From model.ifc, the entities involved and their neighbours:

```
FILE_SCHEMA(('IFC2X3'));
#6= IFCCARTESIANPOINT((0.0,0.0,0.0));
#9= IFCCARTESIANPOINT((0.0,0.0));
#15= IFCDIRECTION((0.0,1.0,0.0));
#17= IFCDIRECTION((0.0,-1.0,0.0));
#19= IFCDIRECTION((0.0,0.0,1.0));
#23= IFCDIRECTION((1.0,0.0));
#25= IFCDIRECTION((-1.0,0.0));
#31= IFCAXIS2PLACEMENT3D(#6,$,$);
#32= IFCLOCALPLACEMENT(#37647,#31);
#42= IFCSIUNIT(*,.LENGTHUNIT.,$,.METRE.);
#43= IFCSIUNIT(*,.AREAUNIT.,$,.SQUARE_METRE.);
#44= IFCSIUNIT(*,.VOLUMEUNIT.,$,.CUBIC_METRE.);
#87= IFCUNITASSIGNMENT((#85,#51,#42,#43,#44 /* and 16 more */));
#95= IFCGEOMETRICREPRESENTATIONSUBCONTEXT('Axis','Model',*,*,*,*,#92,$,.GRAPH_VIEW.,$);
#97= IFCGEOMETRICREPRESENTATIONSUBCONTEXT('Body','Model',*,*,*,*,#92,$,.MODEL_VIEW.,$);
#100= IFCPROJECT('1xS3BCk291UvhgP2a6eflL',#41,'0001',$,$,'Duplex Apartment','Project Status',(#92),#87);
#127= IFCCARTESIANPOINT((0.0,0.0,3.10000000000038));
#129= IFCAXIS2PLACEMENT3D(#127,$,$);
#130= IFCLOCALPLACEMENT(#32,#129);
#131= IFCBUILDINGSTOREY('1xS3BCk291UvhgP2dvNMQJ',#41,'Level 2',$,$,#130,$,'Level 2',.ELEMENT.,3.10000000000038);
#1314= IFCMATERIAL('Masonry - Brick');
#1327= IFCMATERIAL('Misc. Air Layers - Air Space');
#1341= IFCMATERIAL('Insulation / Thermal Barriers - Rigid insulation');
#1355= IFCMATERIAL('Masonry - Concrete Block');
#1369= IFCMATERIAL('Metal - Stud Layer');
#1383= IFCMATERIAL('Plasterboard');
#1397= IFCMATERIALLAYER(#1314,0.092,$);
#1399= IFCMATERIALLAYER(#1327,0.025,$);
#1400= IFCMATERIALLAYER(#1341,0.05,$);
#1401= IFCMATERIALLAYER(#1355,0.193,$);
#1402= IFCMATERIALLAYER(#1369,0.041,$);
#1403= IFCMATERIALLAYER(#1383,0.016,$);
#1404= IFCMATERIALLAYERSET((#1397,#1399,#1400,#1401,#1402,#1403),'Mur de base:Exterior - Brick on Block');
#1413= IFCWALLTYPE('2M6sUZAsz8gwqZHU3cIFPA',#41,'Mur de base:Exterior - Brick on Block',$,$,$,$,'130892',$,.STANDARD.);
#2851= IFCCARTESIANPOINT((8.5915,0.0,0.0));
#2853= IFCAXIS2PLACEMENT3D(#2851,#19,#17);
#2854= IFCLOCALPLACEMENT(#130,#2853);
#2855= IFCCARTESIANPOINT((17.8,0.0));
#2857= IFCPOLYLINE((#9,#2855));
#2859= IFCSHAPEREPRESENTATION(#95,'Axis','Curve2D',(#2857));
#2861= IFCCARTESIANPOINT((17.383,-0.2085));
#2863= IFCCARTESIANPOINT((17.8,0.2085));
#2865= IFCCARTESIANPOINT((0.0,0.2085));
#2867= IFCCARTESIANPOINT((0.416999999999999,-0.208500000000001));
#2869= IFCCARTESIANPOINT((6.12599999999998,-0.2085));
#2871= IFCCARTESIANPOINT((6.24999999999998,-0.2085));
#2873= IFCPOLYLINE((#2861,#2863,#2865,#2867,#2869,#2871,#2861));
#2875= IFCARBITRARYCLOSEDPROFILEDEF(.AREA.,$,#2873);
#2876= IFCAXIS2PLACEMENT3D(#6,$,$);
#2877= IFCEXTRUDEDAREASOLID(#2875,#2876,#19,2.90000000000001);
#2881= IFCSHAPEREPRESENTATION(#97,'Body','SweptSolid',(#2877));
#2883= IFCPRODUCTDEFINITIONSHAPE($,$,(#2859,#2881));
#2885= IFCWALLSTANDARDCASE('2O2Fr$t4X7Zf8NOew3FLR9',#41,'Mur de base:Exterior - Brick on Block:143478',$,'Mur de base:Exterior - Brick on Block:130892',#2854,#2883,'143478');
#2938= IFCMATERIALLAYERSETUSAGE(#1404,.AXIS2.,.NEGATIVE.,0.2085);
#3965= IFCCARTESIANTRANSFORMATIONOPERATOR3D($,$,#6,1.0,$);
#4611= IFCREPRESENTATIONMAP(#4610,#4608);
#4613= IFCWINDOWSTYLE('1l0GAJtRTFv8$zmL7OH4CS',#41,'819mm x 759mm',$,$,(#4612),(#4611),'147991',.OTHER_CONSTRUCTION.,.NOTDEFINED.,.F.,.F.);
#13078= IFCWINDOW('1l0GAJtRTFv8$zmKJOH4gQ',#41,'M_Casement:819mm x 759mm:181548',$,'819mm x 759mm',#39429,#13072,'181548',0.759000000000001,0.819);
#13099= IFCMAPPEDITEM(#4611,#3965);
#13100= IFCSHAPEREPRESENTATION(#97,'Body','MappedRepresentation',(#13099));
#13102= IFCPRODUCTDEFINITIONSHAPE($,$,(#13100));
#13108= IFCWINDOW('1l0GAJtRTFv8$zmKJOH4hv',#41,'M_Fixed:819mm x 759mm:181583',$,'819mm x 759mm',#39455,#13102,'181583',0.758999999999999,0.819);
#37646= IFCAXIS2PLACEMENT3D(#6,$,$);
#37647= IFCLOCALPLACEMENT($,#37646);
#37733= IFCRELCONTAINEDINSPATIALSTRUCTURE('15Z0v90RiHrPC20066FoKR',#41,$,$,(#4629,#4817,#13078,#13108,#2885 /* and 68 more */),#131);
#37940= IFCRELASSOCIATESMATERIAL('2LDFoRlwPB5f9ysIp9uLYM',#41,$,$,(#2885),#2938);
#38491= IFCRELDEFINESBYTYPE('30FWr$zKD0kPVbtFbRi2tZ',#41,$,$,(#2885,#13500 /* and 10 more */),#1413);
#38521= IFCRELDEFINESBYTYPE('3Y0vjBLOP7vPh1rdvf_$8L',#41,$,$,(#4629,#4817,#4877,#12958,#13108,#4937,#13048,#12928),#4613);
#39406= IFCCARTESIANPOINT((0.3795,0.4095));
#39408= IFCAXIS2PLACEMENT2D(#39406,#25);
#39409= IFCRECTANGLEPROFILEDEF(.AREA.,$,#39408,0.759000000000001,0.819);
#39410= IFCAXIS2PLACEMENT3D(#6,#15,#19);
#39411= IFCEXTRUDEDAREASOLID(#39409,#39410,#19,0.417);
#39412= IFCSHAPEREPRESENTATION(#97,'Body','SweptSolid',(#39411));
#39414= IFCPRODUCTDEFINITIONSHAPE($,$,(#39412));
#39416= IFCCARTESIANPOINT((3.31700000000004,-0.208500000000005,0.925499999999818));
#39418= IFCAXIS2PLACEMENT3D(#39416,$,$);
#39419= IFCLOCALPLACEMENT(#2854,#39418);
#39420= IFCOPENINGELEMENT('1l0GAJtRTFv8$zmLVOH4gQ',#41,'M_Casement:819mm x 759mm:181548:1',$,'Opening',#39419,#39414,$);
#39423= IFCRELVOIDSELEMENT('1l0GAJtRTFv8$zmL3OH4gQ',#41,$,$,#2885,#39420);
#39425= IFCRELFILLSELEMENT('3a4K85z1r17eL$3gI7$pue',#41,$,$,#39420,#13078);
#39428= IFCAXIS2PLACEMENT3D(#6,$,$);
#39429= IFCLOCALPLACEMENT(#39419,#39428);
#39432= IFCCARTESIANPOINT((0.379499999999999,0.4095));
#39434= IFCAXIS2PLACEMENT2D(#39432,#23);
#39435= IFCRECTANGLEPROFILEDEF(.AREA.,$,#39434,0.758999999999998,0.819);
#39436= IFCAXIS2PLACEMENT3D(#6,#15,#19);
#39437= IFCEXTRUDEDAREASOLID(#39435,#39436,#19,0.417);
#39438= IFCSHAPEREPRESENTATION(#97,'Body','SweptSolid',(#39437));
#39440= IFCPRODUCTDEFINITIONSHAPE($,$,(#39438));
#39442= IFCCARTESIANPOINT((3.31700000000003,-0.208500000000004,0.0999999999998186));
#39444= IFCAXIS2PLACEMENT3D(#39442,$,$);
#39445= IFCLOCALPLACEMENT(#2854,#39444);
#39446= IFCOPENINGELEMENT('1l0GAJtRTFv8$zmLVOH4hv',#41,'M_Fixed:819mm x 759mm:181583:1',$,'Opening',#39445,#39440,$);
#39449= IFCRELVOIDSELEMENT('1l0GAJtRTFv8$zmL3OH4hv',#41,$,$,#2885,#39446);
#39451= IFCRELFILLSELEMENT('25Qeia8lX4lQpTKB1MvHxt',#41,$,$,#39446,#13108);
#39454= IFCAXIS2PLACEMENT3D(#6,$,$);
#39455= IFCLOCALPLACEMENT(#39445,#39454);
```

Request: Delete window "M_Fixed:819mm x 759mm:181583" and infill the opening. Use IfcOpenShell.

```python
import ifcopenshell
import ifcopenshell.api.feature
import ifcopenshell.api.root
import ifcopenshell.geom
import ifcopenshell.util.shape

model = ifcopenshell.open("model.ifc")
settings = ifcopenshell.geom.settings()


def volume(element):
    """Net volume in cubic metres, openings subtracted."""
    shape = ifcopenshell.geom.create_shape(settings, element)
    return ifcopenshell.util.shape.get_volume(shape.geometry)


window = model.by_guid("1l0GAJtRTFv8$zmKJOH4hv")
opening = window.FillsVoids[0].RelatingOpeningElement
wall = opening.VoidsElements[0].RelatingBuildingElement
before = volume(wall)

ifcopenshell.api.root.remove_product(model, product=window)
ifcopenshell.api.feature.remove_feature(model, feature=opening)

after = volume(wall)

print(f"wall volume {before:.3f} -> {after:.3f} m3")

model.write("model_rev.ifc")
```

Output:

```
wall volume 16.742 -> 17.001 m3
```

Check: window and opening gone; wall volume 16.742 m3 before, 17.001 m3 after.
